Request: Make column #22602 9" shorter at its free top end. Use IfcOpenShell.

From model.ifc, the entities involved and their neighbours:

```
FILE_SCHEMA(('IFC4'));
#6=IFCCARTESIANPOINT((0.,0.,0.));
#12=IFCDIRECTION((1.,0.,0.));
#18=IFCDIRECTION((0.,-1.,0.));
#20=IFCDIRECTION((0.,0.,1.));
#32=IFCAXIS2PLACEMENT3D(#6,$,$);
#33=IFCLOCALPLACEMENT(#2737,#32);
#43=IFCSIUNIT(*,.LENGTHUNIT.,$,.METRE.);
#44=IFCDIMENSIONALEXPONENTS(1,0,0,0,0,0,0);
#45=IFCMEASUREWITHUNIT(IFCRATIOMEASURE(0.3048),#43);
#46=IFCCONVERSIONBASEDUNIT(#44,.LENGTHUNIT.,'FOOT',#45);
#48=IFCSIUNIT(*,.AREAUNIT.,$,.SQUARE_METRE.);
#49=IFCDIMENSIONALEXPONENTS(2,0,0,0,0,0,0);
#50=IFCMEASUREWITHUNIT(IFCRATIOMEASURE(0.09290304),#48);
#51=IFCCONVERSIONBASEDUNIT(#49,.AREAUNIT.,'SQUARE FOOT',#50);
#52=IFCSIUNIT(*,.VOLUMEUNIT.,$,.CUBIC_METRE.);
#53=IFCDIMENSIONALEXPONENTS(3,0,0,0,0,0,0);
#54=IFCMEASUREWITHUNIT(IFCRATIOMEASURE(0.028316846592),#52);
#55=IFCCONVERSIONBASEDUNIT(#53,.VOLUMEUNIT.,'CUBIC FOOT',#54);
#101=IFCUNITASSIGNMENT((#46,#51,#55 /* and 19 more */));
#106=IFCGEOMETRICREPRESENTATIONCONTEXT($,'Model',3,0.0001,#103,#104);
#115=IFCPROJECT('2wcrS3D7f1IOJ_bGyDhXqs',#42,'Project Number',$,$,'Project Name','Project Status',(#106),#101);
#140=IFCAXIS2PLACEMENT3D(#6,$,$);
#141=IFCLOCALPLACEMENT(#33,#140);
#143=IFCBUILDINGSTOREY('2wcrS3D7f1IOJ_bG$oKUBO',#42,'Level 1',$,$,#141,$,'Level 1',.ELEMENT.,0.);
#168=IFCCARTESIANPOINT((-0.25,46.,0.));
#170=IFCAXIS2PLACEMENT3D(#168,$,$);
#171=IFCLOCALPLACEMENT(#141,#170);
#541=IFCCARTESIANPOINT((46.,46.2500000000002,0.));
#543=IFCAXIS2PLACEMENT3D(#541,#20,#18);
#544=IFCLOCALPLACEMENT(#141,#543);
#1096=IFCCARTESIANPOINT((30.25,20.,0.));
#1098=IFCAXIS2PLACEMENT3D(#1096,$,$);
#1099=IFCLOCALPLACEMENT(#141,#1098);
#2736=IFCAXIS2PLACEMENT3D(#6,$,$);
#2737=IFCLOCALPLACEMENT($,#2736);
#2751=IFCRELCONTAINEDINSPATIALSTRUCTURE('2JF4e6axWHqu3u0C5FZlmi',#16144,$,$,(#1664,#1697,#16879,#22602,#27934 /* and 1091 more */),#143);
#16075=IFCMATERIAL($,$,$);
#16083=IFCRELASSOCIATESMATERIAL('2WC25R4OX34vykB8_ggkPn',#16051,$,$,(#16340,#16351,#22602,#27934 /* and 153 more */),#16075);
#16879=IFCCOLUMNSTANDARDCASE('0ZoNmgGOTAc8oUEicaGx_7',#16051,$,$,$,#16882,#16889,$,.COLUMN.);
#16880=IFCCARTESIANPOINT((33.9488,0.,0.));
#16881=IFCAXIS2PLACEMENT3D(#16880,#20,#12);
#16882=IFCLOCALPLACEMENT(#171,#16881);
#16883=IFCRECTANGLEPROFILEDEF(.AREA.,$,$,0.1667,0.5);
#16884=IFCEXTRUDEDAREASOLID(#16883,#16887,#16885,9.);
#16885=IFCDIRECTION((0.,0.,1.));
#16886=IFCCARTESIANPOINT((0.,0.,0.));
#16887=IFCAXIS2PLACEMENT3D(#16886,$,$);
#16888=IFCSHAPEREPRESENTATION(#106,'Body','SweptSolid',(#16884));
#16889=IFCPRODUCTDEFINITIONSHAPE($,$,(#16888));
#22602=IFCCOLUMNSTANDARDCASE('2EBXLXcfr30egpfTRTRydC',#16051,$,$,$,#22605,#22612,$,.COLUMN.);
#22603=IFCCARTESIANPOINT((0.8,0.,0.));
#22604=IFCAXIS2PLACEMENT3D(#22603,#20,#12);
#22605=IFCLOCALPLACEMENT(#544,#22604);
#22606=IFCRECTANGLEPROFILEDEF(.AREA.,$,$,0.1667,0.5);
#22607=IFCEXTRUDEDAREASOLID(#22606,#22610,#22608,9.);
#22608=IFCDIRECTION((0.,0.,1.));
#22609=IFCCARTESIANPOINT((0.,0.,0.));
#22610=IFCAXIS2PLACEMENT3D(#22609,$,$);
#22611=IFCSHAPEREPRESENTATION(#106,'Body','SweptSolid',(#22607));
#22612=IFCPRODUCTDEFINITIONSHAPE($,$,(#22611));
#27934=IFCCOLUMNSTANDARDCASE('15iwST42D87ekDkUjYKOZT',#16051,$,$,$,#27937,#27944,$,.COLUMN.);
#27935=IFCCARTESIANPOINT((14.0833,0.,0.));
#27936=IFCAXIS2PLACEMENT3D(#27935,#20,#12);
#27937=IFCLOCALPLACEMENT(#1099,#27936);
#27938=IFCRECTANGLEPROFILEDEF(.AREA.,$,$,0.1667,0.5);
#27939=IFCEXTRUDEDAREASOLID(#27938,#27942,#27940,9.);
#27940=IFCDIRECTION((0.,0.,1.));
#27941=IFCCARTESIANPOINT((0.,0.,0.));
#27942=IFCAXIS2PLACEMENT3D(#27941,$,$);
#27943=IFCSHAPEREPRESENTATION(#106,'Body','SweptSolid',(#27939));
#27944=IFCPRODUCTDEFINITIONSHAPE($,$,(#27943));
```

```python
import ifcopenshell
import ifcopenshell.util.unit

model = ifcopenshell.open("model.ifc")
unit_scale = ifcopenshell.util.unit.calculate_unit_scale(model)

member = model.by_id(22602)
change = -9 * 0.0254 / unit_scale

# The extrusion runs towards the end named, so only its depth changes.
body = next(r for r in member.Representation.Representations if r.RepresentationIdentifier == "Body")
solid = body.Items[0]
old_length = solid.Depth
solid.Depth += change

print(f"length {old_length:g} -> {solid.Depth:g}")

model.write("model_updated.ifc")
```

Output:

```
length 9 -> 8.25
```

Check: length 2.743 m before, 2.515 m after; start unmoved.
